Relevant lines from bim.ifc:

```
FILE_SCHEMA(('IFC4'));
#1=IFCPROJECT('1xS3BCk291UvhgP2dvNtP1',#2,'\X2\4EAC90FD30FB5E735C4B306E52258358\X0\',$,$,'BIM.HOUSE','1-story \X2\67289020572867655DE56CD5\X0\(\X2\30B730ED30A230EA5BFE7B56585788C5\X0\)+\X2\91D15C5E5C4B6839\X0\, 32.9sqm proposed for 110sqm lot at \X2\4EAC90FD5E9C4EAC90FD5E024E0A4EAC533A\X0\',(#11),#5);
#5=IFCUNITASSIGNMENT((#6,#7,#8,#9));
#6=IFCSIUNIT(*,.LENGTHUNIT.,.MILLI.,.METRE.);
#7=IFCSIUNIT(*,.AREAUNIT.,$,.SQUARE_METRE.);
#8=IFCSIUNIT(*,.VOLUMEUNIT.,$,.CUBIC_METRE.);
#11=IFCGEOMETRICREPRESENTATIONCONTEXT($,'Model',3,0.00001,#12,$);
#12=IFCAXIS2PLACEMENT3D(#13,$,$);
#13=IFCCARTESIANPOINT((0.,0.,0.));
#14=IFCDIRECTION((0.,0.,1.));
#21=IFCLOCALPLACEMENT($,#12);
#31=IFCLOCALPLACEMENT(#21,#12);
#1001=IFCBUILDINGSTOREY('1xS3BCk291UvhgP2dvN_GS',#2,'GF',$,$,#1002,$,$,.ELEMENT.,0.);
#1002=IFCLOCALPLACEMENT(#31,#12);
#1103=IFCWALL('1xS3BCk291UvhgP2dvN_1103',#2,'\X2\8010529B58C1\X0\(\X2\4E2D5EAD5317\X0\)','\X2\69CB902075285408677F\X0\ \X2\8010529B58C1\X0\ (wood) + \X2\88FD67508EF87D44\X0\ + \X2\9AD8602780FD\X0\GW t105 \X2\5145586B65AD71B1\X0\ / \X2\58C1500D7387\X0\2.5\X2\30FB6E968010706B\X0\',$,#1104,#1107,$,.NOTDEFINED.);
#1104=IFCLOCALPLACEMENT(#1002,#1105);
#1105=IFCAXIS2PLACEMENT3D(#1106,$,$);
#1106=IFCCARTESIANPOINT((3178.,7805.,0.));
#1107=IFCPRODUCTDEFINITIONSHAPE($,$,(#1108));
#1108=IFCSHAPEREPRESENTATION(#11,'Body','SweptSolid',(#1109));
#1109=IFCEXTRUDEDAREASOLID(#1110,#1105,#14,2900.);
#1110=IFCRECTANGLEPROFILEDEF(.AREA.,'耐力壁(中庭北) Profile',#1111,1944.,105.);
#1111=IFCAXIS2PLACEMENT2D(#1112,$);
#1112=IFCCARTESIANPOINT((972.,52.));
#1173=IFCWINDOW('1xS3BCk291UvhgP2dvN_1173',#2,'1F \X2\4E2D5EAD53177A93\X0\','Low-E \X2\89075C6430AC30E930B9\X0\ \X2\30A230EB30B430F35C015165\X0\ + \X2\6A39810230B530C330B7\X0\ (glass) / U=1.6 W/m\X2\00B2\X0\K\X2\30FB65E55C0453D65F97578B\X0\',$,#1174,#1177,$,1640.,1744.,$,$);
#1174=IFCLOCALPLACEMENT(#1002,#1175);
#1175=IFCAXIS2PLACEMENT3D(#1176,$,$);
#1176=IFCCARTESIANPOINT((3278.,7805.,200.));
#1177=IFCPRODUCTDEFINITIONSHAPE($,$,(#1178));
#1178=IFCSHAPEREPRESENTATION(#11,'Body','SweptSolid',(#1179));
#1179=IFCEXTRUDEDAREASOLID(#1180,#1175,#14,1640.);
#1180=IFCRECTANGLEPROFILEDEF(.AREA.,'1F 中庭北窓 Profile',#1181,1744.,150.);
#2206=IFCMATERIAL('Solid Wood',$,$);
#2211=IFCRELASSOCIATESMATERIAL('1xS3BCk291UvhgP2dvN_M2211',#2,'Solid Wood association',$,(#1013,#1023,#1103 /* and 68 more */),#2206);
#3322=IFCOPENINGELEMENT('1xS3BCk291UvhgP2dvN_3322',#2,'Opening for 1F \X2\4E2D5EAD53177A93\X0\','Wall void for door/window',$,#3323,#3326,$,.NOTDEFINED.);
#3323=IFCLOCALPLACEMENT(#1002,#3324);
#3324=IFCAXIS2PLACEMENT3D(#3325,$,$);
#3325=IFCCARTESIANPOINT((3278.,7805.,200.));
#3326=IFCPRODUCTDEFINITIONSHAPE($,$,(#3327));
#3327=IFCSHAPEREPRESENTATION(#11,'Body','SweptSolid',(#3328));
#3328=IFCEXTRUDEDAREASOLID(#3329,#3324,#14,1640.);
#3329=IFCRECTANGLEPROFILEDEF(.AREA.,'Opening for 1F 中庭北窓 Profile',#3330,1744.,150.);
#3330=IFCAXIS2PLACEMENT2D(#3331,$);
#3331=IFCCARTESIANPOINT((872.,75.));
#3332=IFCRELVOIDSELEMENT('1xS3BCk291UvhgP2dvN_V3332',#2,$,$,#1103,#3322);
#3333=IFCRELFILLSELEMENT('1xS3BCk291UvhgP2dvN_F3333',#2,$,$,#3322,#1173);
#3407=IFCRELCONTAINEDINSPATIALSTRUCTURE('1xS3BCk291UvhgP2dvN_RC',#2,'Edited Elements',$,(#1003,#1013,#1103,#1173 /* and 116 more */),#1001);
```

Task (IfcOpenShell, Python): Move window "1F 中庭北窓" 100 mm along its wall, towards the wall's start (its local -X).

```python
import ifcopenshell
import ifcopenshell.api.geometry
import ifcopenshell.util.placement
import ifcopenshell.util.unit

model = ifcopenshell.open("bim.ifc")
unit_scale = ifcopenshell.util.unit.calculate_unit_scale(model)

window = model.by_guid("1xS3BCk291UvhgP2dvN_1173")
opening = window.FillsVoids[0].RelatingOpeningElement
wall = opening.VoidsElements[0].RelatingBuildingElement

wall_matrix = ifcopenshell.util.placement.get_local_placement(wall.ObjectPlacement)
shift = wall_matrix[:3, 0] * -0.1 / unit_scale
before = ifcopenshell.util.placement.get_local_placement(window.ObjectPlacement)[:3, 3].copy()

# The window is not placed relative to its opening, so move both.
for product in (opening, window):
    matrix = ifcopenshell.util.placement.get_local_placement(product.ObjectPlacement)
    matrix[:3, 3] += shift
    ifcopenshell.api.geometry.edit_object_placement(model, product=product, matrix=matrix, is_si=False)

after = ifcopenshell.util.placement.get_local_placement(window.ObjectPlacement)[:3, 3]
print("window moved by", (after - before).round(3) + 0.0)

model.write("bim_updated.ifc")
```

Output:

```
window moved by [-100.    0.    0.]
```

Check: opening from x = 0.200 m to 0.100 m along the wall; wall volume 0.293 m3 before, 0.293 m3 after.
